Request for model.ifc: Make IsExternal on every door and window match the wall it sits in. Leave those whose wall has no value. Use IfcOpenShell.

First a look at what the model holds.

```python
import ifcopenshell
import ifcopenshell.util.element

model = ifcopenshell.open("model.ifc")
print(model.schema)
seen = {}
for e in model.by_type("IfcDoor") + model.by_type("IfcWindow"):
    if not e.FillsVoids:
        continue
    host = e.FillsVoids[0].RelatingOpeningElement.VoidsElements[0].RelatingBuildingElement
    own = ifcopenshell.util.element.get_pset(e, f"Pset_{e.is_a()[3:].removesuffix('StandardCase')}Common", "IsExternal")
    wall = ifcopenshell.util.element.get_pset(host, "Pset_WallCommon", "IsExternal")
    seen[e.is_a(), own, wall] = seen.get((e.is_a(), own, wall), 0) + 1
for (cls, own, wall), count in sorted(seen.items(), key=str):
    print(count, cls, "IsExternal:", own, "| host wall:", wall)
```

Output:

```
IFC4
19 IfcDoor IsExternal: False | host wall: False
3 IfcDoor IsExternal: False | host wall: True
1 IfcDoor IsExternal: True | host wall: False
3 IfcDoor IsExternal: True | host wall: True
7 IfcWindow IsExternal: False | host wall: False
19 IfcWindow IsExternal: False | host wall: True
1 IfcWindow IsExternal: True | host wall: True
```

```python
import ifcopenshell
import ifcopenshell.api.pset
import ifcopenshell.util.element

model = ifcopenshell.open("model.ifc")

count = 0
for ifc_class, pset_name in (("IfcDoor", "Pset_DoorCommon"), ("IfcWindow", "Pset_WindowCommon")):
    for e in model.by_type(ifc_class):
        if not e.FillsVoids:
            continue
        host = e.FillsVoids[0].RelatingOpeningElement.VoidsElements[0].RelatingBuildingElement
        external = ifcopenshell.util.element.get_pset(host, "Pset_WallCommon", "IsExternal")
        if external is None or ifcopenshell.util.element.get_pset(e, pset_name, "IsExternal") == external:
            continue
        pset = ifcopenshell.api.pset.add_pset(model, product=e, name=pset_name)
        ifcopenshell.api.pset.edit_pset(model, pset=pset, properties={"IsExternal": external})
        count += 1

print(count, "updated")

model.write("model_v2.ifc")
```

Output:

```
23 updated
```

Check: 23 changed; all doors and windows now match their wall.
